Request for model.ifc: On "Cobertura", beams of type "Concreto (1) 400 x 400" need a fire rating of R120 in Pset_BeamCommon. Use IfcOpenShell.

First a look at what the model holds.

```python
import ifcopenshell
import ifcopenshell.util.element

model = ifcopenshell.open("model.ifc")
print(model.schema)
storey = next(s for s in model.by_type("IfcBuildingStorey") if s.Name == "Cobertura")
beams = [e for e in ifcopenshell.util.element.get_decomposition(storey) if e.is_a("IfcBeam")]
seen = {}
for e in beams:
    element_type = ifcopenshell.util.element.get_type(e)
    key = (element_type.Name if element_type != e and element_type else None, ifcopenshell.util.element.get_pset(e, "Pset_BeamCommon", "FireRating"))
    seen[key] = seen.get(key, 0) + 1
for (name, value), count in sorted(seen.items(), key=str):
    print(count, "x", name, "|", value)
```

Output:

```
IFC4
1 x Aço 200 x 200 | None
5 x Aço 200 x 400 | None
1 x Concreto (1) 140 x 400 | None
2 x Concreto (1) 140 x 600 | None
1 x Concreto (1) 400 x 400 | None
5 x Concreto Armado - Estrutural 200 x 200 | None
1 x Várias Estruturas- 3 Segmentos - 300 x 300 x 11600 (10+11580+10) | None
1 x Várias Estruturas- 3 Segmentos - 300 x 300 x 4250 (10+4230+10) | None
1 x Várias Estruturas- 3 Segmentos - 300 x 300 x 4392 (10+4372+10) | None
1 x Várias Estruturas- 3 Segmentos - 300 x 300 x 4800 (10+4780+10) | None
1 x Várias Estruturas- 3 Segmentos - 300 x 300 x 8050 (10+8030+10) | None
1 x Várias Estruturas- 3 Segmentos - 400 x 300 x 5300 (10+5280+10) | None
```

```python
import ifcopenshell
import ifcopenshell.api.pset
import ifcopenshell.util.element

model = ifcopenshell.open("model.ifc")

storey = next(s for s in model.by_type("IfcBuildingStorey") if s.Name == "Cobertura")
beams = [e for e in ifcopenshell.util.element.get_decomposition(storey) if e.is_a("IfcBeam")]

count = 0
for e in beams:
    element_type = ifcopenshell.util.element.get_type(e)
    if element_type in (None, e) or element_type.Name != "Concreto (1) 400 x 400":
        continue
    # add_pset returns the element's existing set when there is one.
    pset = ifcopenshell.api.pset.add_pset(model, product=e, name="Pset_BeamCommon")
    ifcopenshell.api.pset.edit_pset(model, pset=pset, properties={"FireRating": "R120"})
    count += 1

print(count, "beams updated")

model.write("model-out.ifc")
```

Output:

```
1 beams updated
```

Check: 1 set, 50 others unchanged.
